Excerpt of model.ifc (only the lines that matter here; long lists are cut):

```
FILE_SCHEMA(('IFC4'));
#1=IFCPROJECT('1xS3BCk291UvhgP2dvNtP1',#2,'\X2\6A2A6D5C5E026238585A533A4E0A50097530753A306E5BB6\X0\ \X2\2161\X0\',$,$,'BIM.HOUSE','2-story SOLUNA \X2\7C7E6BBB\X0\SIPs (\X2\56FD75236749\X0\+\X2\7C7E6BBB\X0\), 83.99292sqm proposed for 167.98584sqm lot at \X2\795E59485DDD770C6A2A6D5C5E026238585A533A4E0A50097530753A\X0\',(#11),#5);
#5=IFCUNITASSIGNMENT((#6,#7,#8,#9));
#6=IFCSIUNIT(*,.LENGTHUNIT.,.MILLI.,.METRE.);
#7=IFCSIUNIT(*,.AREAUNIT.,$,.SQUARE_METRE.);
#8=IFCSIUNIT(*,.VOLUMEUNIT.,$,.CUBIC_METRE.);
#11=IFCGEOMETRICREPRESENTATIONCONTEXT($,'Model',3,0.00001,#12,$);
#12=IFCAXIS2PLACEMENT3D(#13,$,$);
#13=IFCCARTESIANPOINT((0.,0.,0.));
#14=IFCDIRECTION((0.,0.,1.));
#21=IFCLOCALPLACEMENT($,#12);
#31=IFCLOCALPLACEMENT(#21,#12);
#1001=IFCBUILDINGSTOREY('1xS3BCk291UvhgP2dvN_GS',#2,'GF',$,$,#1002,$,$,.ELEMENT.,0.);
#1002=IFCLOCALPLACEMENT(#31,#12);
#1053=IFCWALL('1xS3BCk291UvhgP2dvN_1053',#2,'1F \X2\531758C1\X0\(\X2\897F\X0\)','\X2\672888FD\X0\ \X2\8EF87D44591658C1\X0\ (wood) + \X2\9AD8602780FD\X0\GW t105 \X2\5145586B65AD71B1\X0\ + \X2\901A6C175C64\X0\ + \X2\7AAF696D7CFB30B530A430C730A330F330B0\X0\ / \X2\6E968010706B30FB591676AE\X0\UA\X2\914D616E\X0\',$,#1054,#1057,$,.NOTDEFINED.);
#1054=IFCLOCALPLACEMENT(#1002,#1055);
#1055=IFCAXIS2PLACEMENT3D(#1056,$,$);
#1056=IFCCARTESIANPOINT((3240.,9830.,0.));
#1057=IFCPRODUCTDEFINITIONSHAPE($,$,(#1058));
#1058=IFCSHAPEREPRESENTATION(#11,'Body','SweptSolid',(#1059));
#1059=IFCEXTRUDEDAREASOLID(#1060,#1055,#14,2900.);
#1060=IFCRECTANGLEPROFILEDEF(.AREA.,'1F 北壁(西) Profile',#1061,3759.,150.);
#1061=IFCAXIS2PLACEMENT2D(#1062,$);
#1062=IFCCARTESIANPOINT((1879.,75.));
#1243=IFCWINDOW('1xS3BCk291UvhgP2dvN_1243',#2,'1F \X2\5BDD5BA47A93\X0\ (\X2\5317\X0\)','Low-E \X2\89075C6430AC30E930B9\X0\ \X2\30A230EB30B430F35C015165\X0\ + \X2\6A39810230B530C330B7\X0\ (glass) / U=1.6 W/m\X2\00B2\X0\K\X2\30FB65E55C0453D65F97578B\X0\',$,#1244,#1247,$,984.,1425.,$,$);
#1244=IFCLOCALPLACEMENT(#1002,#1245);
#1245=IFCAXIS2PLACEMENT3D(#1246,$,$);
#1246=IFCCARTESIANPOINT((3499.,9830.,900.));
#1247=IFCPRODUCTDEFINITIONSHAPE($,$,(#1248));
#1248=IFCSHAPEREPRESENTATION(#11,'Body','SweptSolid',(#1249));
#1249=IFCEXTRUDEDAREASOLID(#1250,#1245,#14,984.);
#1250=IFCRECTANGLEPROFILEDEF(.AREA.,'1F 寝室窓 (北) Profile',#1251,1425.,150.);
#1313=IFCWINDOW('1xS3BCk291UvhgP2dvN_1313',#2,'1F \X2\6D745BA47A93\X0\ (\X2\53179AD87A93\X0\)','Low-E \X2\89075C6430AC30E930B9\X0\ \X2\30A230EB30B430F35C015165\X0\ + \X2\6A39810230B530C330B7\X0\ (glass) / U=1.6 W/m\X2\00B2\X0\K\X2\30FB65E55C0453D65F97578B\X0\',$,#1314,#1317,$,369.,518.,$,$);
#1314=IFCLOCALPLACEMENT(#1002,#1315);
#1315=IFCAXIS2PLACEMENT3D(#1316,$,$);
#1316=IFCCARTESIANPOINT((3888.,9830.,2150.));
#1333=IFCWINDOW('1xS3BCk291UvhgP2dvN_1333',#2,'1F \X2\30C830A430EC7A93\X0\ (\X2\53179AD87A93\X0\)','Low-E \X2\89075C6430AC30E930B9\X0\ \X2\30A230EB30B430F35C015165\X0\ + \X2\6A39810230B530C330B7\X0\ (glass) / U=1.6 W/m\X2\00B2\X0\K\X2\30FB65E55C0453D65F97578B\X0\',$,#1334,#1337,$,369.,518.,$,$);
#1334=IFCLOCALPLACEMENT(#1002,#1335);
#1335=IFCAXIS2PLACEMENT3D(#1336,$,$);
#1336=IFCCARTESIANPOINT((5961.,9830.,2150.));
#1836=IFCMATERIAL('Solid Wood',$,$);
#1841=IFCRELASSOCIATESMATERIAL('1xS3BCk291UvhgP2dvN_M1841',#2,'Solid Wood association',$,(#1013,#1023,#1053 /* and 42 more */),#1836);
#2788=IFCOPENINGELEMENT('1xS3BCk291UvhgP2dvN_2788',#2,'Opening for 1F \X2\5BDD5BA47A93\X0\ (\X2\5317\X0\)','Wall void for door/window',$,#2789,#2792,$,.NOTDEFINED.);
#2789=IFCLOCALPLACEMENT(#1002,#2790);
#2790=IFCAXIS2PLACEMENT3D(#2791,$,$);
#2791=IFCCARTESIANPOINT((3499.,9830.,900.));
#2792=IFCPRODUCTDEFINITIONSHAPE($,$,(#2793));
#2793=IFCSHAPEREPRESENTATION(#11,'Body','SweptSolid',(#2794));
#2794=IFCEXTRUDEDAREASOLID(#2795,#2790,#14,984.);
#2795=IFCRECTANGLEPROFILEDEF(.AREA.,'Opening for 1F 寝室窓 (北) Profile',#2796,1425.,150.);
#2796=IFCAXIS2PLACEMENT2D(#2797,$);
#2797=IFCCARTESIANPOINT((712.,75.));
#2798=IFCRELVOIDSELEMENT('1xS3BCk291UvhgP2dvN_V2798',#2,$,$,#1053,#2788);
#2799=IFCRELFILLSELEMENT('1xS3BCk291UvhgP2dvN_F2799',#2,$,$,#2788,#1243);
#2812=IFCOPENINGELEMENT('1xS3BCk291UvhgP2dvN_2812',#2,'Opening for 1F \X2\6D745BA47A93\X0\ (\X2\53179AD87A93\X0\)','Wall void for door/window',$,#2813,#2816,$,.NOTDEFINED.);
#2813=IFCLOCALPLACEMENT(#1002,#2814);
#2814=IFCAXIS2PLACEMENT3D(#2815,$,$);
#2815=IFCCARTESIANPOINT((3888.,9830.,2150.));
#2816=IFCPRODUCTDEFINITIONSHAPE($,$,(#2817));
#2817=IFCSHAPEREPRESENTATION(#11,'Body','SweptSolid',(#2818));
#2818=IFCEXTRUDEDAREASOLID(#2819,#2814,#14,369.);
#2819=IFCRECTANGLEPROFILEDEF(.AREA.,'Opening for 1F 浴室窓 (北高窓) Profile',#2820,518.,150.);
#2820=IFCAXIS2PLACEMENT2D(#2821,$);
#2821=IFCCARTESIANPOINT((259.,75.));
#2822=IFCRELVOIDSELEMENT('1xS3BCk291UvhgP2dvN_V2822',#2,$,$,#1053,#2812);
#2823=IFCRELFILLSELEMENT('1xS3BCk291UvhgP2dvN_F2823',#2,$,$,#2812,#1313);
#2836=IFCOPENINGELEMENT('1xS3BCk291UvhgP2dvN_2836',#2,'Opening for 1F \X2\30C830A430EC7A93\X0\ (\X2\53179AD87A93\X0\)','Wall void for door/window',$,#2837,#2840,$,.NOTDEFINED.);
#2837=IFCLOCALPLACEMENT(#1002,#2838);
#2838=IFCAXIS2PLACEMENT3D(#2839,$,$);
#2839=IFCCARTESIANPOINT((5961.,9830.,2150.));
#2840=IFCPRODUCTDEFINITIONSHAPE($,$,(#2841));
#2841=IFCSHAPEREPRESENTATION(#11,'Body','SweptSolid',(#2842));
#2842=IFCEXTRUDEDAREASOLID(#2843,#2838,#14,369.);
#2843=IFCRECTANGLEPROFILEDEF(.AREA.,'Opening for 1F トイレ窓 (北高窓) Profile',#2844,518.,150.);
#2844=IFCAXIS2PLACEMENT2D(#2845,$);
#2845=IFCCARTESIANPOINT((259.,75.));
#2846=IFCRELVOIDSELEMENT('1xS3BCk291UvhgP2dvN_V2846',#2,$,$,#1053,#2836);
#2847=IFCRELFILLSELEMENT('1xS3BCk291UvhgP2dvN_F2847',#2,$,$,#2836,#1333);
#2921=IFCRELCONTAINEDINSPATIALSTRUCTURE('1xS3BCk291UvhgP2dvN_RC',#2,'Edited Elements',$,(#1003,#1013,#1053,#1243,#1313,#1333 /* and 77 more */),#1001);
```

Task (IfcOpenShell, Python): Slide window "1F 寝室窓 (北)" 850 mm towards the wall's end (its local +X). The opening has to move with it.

```python
import ifcopenshell
import ifcopenshell.api.geometry
import ifcopenshell.util.placement
import ifcopenshell.util.unit

model = ifcopenshell.open("model.ifc")
unit_scale = ifcopenshell.util.unit.calculate_unit_scale(model)

window = model.by_guid("1xS3BCk291UvhgP2dvN_1243")
opening = window.FillsVoids[0].RelatingOpeningElement
wall = opening.VoidsElements[0].RelatingBuildingElement

wall_matrix = ifcopenshell.util.placement.get_local_placement(wall.ObjectPlacement)
shift = wall_matrix[:3, 0] * 0.85 / unit_scale
before = ifcopenshell.util.placement.get_local_placement(window.ObjectPlacement)[:3, 3].copy()

# The window is not placed relative to its opening, so move both.
for product in (opening, window):
    matrix = ifcopenshell.util.placement.get_local_placement(product.ObjectPlacement)
    matrix[:3, 3] += shift
    ifcopenshell.api.geometry.edit_object_placement(model, product=product, matrix=matrix, is_si=False)

after = ifcopenshell.util.placement.get_local_placement(window.ObjectPlacement)[:3, 3]
print("window moved by", (after - before).round(3) + 0.0)

model.write("model-out.ifc")
```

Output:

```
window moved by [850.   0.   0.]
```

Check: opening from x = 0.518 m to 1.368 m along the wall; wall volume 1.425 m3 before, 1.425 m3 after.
